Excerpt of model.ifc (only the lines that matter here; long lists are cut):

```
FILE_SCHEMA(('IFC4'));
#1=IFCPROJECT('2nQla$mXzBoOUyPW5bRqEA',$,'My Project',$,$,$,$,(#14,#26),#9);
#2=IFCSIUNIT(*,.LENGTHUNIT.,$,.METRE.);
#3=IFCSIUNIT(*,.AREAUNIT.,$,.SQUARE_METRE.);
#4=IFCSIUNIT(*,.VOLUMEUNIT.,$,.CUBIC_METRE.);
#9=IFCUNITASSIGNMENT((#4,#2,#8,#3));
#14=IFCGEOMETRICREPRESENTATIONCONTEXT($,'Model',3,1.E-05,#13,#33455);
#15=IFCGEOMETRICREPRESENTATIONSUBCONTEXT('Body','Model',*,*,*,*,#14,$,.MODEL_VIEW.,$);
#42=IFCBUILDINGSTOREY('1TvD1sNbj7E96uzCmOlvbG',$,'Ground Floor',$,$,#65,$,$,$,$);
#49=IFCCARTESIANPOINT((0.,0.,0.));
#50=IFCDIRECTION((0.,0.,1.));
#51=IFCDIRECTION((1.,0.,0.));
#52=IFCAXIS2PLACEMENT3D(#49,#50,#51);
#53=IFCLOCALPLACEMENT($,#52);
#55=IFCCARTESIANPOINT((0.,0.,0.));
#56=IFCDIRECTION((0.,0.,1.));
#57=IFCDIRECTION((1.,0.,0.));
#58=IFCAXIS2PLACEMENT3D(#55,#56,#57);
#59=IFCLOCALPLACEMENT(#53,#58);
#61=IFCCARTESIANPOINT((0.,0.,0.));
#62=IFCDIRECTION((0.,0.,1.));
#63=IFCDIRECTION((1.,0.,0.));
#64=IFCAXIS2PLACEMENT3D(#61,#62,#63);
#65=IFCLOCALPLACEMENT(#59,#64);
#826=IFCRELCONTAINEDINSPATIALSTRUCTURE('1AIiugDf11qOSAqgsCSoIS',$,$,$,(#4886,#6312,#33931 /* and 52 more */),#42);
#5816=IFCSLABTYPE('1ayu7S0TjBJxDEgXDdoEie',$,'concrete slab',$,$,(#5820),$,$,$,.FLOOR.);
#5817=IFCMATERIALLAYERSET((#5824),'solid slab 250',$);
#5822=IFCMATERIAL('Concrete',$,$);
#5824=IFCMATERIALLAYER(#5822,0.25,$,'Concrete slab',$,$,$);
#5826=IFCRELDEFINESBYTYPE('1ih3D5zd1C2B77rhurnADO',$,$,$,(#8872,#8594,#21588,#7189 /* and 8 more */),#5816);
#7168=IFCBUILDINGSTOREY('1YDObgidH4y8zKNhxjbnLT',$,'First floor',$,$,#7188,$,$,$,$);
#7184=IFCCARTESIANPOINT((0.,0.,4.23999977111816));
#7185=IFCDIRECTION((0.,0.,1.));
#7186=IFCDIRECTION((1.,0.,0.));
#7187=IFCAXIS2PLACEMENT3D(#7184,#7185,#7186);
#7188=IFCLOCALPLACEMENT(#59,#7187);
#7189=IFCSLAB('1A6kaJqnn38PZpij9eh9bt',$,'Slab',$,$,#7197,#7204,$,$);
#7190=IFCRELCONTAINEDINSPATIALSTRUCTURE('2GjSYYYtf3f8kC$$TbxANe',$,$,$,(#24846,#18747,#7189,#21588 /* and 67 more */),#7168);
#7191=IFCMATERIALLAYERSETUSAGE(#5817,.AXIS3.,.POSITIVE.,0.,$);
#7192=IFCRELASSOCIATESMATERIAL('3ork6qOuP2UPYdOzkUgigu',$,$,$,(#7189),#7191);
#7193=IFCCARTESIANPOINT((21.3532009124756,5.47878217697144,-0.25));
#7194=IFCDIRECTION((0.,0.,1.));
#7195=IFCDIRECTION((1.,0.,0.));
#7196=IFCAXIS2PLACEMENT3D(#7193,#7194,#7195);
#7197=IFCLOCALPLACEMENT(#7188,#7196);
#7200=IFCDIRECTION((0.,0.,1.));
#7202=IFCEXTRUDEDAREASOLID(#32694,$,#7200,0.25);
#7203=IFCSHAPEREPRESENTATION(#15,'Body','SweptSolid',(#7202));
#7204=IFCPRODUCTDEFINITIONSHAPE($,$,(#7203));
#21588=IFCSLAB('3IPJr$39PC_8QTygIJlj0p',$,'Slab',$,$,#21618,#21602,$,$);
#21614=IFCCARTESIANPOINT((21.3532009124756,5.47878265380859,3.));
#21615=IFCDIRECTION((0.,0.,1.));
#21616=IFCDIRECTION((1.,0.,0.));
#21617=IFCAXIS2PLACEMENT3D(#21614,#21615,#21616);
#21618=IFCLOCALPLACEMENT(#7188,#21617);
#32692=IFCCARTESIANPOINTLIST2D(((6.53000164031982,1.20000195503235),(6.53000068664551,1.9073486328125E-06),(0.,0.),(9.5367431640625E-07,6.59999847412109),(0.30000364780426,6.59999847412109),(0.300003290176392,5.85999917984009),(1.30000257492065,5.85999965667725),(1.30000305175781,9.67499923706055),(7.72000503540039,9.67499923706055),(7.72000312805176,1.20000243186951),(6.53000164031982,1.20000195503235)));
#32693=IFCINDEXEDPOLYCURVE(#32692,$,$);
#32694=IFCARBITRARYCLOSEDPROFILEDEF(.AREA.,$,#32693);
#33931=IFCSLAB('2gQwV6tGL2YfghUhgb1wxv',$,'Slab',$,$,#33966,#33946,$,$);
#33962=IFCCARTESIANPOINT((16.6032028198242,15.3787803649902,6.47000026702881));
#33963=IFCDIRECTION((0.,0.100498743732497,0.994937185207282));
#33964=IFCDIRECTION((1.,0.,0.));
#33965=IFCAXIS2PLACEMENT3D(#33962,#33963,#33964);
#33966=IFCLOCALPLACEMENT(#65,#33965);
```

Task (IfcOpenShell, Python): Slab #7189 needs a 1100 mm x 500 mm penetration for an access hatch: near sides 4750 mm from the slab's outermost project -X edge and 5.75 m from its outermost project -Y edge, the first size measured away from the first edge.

```python
import numpy as np
import ifcopenshell
import ifcopenshell.api.feature
import ifcopenshell.api.geometry
import ifcopenshell.api.root
import ifcopenshell.geom
import ifcopenshell.util.placement
import ifcopenshell.util.representation
import ifcopenshell.util.shape
import ifcopenshell.util.unit

model = ifcopenshell.open("model.ifc")
unit_scale = ifcopenshell.util.unit.calculate_unit_scale(model)
settings = ifcopenshell.geom.settings()


def volume(element):
    """Net volume in cubic metres, openings subtracted."""
    shape = ifcopenshell.geom.create_shape(settings, element)
    return ifcopenshell.util.shape.get_volume(shape.geometry)


slab = model.by_guid("1A6kaJqnn38PZpij9eh9bt")
before = volume(slab)

# Extent in the slab's own axes, in metres. The edges named are its -X and -Y sides.
slab_shape = ifcopenshell.geom.create_shape(settings, slab)
vertices = ifcopenshell.util.shape.get_vertices(slab_shape.geometry)
x_min, y_min, bottom = vertices.min(axis=0)
top = vertices[:, 2].max()

opening = ifcopenshell.api.root.create_entity(model, ifc_class="IfcOpeningElement", name="Access hatch opening", predefined_type="OPENING")
context = ifcopenshell.util.representation.get_context(model, "Model", "Body", "MODEL_VIEW")
width, depth = 1.1, 0.5
outline = [(0.0, 0.0), (width, 0.0), (width, depth), (0.0, depth), (0.0, 0.0)]
# Overshoot both faces by 50 mm so the cut is clean.
shape = ifcopenshell.api.geometry.add_slab_representation(
    model, context=context, depth=top - bottom + 0.1, polyline=outline
)
ifcopenshell.api.geometry.assign_representation(model, product=opening, representation=shape)

matrix = ifcopenshell.util.placement.get_local_placement(slab.ObjectPlacement)
matrix[:, 3] = matrix @ np.append(np.array([x_min + 4.75, y_min + 5.75, bottom - 0.05]) / unit_scale, 1.0)
ifcopenshell.api.geometry.edit_object_placement(model, product=opening, matrix=matrix, is_si=False)
ifcopenshell.api.feature.add_feature(model, feature=opening, element=slab)

after = volume(slab)

print(f"slab volume {before:.3f} -> {after:.3f} m3")

model.write("model_v2.ifc")
```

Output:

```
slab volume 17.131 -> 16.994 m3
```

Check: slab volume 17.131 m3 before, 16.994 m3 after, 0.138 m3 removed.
